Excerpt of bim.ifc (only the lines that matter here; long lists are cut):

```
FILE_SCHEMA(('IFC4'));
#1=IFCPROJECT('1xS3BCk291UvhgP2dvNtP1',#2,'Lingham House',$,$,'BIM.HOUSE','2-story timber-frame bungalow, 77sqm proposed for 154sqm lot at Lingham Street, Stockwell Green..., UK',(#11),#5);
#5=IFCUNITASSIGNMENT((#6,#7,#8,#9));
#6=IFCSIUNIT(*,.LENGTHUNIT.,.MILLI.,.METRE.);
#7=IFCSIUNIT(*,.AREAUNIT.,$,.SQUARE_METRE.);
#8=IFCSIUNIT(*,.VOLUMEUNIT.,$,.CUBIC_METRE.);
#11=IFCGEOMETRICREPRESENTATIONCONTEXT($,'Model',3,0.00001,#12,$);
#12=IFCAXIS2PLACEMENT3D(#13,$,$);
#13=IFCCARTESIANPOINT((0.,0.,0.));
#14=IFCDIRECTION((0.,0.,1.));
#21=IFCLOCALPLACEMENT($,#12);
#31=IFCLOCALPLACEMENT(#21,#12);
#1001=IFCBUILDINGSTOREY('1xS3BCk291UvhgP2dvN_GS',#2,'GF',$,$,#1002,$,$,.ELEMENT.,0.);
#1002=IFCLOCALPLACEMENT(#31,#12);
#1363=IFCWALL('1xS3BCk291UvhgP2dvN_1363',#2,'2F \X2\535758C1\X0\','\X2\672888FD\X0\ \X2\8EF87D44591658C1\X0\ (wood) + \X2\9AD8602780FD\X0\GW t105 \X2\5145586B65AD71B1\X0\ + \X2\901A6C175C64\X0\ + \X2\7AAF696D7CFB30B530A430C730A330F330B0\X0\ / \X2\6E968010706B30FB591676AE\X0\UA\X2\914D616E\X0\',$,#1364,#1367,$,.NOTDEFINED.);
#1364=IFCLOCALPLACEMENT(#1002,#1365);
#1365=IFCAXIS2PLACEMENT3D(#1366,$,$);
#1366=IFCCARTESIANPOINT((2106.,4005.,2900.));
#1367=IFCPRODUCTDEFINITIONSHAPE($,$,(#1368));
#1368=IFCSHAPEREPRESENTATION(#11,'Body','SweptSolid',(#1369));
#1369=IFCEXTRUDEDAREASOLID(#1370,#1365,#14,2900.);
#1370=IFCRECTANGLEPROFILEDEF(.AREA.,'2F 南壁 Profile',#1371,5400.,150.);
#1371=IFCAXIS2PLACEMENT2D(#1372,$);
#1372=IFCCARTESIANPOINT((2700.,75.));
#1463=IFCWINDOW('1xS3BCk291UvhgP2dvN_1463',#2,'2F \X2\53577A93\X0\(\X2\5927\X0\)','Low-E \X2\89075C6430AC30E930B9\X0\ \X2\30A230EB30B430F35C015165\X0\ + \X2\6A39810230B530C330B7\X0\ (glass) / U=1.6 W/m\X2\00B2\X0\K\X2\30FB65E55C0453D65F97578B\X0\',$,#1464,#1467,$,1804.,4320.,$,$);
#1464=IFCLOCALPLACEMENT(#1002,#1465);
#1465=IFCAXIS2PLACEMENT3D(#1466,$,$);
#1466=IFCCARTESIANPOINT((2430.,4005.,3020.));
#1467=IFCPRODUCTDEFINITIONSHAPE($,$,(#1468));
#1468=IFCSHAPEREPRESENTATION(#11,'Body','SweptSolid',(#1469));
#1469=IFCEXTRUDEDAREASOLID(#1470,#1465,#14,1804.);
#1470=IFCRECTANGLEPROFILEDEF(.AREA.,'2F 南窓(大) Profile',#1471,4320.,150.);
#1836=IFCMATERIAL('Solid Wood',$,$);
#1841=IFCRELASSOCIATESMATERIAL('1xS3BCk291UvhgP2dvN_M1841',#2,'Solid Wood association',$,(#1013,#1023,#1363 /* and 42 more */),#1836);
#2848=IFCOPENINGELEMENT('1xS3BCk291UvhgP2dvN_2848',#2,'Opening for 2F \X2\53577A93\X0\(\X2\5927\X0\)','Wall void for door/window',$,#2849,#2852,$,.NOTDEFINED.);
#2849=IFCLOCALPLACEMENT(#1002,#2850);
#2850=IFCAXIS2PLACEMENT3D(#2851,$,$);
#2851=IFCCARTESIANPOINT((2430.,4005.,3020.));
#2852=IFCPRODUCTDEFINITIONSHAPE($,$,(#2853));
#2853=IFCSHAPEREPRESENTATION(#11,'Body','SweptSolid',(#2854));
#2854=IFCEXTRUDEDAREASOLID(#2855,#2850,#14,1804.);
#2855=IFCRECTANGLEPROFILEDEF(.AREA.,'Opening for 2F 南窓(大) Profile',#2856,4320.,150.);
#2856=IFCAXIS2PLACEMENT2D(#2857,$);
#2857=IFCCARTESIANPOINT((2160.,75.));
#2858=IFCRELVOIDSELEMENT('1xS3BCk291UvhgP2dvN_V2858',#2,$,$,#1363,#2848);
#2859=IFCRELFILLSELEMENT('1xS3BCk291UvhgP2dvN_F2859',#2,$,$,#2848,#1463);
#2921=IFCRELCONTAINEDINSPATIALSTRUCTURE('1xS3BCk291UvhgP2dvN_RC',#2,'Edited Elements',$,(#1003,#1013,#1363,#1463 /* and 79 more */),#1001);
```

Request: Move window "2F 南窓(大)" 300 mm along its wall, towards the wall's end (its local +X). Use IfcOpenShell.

```python
import ifcopenshell
import ifcopenshell.api.geometry
import ifcopenshell.util.placement

model = ifcopenshell.open("bim.ifc")

window = model.by_guid("1xS3BCk291UvhgP2dvN_1463")
opening = window.FillsVoids[0].RelatingOpeningElement
wall = opening.VoidsElements[0].RelatingBuildingElement

wall_matrix = ifcopenshell.util.placement.get_local_placement(wall.ObjectPlacement)
shift = wall_matrix[:3, 0] * 300.0
before = ifcopenshell.util.placement.get_local_placement(window.ObjectPlacement)[:3, 3].copy()

# The window is not placed relative to its opening, so move both.
for product in (opening, window):
    matrix = ifcopenshell.util.placement.get_local_placement(product.ObjectPlacement)
    matrix[:3, 3] += shift
    ifcopenshell.api.geometry.edit_object_placement(model, product=product, matrix=matrix, is_si=False)

after = ifcopenshell.util.placement.get_local_placement(window.ObjectPlacement)[:3, 3]
print("window moved by", (after - before).round(3) + 0.0)

model.write("bim_updated.ifc")
```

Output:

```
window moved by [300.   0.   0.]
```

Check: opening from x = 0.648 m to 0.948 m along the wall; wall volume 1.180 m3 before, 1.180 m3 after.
